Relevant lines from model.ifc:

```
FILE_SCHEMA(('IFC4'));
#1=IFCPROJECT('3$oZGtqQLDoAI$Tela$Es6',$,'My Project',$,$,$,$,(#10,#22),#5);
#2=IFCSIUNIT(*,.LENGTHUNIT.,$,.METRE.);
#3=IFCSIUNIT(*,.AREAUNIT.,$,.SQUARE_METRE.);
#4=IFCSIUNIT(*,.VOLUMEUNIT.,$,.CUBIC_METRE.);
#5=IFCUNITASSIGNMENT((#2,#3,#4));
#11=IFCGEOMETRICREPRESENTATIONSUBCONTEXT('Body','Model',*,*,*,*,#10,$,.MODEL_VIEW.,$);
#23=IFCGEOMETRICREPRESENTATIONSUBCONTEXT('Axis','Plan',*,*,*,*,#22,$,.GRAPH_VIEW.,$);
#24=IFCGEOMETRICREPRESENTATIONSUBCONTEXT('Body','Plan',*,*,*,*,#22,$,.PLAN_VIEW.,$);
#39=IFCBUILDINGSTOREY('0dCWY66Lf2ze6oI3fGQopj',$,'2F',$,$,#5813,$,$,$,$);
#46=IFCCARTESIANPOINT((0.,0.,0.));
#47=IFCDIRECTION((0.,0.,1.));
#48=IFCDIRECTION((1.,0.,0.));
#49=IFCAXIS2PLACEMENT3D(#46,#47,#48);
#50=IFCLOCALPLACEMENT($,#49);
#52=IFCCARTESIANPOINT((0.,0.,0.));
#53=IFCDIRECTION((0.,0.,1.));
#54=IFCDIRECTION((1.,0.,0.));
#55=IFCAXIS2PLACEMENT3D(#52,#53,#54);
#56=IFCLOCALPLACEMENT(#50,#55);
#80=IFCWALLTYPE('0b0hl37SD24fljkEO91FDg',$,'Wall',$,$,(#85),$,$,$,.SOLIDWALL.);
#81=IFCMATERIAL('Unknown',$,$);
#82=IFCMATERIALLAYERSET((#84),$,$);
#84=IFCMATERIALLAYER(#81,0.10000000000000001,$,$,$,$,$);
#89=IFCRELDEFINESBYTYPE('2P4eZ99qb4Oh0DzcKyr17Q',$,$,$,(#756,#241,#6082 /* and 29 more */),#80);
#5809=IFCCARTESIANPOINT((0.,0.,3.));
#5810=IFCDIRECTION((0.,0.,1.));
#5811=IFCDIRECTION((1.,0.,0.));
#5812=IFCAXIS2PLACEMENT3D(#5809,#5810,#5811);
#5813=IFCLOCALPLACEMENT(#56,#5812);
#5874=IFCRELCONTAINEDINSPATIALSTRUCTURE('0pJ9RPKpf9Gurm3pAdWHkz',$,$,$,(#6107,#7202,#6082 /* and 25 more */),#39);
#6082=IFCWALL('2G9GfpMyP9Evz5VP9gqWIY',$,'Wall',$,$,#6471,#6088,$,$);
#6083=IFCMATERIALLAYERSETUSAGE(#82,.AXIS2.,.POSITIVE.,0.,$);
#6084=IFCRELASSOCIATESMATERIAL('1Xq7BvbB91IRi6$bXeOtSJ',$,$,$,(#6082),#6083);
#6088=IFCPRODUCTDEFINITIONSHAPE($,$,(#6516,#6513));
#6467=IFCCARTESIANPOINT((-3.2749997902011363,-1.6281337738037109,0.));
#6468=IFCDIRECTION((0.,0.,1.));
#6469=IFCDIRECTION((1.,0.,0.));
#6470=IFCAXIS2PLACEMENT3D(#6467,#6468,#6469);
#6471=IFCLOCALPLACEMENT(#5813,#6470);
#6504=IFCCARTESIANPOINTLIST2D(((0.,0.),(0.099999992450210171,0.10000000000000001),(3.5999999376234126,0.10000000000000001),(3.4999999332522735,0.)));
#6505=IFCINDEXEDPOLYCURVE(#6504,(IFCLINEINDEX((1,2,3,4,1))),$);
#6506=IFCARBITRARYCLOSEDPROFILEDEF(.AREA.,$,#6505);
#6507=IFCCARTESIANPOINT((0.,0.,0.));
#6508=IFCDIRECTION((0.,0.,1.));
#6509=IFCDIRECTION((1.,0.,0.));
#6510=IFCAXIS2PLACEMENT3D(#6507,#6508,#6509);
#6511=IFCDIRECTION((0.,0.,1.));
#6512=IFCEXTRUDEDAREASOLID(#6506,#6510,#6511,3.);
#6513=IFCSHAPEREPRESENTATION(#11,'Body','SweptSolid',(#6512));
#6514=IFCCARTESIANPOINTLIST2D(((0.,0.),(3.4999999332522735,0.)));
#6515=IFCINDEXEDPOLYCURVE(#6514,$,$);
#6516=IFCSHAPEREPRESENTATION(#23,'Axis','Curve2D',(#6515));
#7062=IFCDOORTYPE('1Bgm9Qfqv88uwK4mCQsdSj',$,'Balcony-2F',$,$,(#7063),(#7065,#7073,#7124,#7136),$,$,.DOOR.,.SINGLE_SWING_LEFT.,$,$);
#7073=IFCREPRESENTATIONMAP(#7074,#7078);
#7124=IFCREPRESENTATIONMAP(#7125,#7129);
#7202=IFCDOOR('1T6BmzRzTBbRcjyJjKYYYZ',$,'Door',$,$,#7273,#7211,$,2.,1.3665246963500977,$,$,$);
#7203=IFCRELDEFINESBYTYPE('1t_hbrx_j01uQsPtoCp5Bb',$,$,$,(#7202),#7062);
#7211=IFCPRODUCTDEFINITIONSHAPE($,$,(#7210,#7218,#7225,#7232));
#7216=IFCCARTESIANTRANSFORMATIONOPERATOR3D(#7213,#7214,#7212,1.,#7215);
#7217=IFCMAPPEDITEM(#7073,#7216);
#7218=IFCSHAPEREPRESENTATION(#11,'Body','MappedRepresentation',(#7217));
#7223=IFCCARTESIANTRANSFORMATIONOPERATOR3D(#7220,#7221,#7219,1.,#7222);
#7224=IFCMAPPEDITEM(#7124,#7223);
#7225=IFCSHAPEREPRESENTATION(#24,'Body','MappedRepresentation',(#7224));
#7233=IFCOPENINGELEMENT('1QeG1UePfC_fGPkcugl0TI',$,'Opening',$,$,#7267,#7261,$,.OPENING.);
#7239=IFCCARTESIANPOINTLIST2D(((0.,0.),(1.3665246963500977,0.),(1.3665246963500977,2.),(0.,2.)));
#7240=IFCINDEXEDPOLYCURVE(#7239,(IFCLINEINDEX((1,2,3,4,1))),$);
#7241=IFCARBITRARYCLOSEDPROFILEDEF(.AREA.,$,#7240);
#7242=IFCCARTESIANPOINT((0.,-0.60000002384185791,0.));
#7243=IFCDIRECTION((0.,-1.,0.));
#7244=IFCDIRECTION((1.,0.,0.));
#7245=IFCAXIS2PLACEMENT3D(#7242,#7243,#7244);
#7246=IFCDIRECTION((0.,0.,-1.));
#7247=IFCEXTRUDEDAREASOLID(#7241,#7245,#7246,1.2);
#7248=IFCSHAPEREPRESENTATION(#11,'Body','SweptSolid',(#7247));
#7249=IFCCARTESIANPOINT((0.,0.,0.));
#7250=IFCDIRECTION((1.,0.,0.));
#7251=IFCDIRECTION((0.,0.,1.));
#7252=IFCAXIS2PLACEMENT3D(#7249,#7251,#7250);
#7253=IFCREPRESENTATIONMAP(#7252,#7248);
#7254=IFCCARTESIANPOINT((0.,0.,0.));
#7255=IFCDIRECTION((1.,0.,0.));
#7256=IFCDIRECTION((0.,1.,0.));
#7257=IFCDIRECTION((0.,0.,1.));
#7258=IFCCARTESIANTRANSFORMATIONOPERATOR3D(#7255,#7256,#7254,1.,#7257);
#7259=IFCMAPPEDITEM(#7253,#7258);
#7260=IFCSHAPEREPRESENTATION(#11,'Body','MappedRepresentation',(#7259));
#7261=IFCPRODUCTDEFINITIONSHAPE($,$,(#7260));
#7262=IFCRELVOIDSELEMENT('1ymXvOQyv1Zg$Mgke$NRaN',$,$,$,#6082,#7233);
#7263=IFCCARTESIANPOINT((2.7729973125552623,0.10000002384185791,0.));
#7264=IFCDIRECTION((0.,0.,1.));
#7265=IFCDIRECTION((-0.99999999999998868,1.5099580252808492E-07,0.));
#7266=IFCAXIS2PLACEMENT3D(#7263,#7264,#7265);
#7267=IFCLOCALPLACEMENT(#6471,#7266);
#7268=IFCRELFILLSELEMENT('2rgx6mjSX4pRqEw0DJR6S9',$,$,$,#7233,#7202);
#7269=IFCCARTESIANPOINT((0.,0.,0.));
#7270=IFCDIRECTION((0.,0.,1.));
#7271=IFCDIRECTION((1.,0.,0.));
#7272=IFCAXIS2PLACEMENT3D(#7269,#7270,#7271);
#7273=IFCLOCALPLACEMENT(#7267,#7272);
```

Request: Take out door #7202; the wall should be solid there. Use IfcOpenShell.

```python
import ifcopenshell
import ifcopenshell.api.feature
import ifcopenshell.api.root
import ifcopenshell.geom
import ifcopenshell.util.shape

model = ifcopenshell.open("model.ifc")
settings = ifcopenshell.geom.settings()


def volume(element):
    """Net volume in cubic metres, openings subtracted."""
    shape = ifcopenshell.geom.create_shape(settings, element)
    return ifcopenshell.util.shape.get_volume(shape.geometry)


door = model.by_id(7202)
opening = door.FillsVoids[0].RelatingOpeningElement
wall = opening.VoidsElements[0].RelatingBuildingElement
before = volume(wall)

ifcopenshell.api.root.remove_product(model, product=door)
ifcopenshell.api.feature.remove_feature(model, feature=opening)

after = volume(wall)

print(f"wall volume {before:.3f} -> {after:.3f} m3")

model.write("model_v2.ifc")
```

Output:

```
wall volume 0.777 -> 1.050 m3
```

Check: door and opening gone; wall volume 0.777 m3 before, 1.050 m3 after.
